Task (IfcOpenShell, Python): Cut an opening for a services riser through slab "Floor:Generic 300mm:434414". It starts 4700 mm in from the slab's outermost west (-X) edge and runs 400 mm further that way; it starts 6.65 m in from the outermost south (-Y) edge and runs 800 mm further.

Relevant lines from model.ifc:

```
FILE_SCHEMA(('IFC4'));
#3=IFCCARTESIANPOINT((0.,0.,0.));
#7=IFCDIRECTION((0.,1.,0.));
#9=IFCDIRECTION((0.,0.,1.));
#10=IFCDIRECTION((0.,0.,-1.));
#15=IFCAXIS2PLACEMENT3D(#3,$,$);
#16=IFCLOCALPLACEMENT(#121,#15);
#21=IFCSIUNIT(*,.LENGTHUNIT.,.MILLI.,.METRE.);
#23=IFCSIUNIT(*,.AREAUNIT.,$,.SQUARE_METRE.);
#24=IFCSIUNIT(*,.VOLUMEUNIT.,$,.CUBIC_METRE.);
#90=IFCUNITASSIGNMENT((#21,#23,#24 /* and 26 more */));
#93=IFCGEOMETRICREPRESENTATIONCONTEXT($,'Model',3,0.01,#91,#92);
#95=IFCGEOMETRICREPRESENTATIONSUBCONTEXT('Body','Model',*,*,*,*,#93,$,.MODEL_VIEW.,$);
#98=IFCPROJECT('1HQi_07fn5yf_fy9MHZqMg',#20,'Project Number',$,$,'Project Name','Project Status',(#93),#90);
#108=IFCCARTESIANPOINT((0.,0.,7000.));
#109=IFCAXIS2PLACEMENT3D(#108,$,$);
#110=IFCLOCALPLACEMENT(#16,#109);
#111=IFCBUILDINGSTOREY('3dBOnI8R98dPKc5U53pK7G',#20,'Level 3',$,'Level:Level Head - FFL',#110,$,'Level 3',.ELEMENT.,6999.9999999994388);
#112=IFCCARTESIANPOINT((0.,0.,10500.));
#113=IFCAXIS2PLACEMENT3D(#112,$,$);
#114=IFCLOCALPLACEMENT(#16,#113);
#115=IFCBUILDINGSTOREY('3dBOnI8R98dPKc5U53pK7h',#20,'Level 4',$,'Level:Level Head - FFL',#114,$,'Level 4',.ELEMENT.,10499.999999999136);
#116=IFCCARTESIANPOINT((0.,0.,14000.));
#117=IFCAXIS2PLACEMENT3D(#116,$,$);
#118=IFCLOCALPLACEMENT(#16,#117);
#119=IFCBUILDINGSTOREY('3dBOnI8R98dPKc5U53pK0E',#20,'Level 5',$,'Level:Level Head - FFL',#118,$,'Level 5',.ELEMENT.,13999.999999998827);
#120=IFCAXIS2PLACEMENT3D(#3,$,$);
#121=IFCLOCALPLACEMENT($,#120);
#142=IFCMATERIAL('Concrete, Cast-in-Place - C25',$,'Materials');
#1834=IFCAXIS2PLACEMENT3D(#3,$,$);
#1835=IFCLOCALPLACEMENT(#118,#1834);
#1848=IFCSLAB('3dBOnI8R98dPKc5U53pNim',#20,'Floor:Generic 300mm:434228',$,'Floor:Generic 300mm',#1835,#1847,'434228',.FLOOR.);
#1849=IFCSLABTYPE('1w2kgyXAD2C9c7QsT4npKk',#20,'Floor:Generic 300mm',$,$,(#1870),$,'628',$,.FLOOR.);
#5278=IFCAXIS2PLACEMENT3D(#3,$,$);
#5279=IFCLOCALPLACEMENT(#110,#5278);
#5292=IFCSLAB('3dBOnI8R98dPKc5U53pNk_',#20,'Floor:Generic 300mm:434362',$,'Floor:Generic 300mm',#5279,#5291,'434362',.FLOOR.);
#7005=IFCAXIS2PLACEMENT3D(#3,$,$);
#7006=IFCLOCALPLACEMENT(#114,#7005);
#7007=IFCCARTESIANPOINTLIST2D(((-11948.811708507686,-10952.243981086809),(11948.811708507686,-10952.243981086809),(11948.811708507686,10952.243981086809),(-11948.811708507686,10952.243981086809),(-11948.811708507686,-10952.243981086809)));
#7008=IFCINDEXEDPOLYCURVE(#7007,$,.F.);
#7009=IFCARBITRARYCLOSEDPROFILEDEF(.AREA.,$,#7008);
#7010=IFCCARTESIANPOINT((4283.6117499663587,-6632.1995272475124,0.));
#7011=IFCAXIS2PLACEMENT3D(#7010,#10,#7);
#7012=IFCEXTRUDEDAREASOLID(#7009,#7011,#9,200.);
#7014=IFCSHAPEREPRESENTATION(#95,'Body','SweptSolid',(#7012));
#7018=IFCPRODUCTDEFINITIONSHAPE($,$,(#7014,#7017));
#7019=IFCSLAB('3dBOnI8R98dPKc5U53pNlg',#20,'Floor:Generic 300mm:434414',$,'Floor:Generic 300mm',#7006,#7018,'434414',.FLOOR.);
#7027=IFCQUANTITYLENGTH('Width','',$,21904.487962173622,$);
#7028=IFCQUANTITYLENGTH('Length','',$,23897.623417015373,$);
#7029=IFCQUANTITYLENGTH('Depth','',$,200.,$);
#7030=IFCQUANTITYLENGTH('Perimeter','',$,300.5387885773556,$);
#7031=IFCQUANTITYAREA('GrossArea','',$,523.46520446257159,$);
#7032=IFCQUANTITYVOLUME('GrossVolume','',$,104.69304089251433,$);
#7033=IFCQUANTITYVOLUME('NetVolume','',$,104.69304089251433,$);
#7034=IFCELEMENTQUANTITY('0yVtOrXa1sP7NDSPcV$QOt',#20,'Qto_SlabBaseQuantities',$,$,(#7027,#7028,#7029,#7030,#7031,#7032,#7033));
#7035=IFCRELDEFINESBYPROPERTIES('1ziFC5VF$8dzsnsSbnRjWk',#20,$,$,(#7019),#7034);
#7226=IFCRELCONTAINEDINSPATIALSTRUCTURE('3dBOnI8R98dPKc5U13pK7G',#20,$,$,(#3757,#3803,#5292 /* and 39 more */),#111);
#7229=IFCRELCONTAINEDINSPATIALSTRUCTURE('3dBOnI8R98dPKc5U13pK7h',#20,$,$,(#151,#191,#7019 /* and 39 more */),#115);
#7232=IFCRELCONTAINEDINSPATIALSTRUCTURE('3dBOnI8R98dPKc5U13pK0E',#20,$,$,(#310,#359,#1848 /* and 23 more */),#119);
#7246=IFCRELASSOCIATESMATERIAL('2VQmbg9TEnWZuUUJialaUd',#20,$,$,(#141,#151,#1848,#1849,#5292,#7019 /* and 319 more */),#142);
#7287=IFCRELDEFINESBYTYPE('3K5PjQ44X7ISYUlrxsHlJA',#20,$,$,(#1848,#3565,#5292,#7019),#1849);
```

```python
import numpy as np
import ifcopenshell
import ifcopenshell.api.feature
import ifcopenshell.api.geometry
import ifcopenshell.api.pset
import ifcopenshell.api.root
import ifcopenshell.geom
import ifcopenshell.util.element
import ifcopenshell.util.placement
import ifcopenshell.util.representation
import ifcopenshell.util.shape
import ifcopenshell.util.unit

model = ifcopenshell.open("model.ifc")
unit_scale = ifcopenshell.util.unit.calculate_unit_scale(model)
volume_scale = ifcopenshell.util.unit.calculate_unit_scale(model, "VOLUMEUNIT")
settings = ifcopenshell.geom.settings()


def volume(element):
    """Net volume in cubic metres, openings subtracted."""
    shape = ifcopenshell.geom.create_shape(settings, element)
    return ifcopenshell.util.shape.get_volume(shape.geometry)


slab = model.by_guid("3dBOnI8R98dPKc5U53pNlg")
before = volume(slab)

# Extent in the slab's own axes, in metres. The edges named are its -X and -Y sides.
slab_shape = ifcopenshell.geom.create_shape(settings, slab)
vertices = ifcopenshell.util.shape.get_vertices(slab_shape.geometry)
x_min, y_min, bottom = vertices.min(axis=0)
top = vertices[:, 2].max()

opening = ifcopenshell.api.root.create_entity(model, ifc_class="IfcOpeningElement", name="Services riser opening", predefined_type="OPENING")
context = ifcopenshell.util.representation.get_context(model, "Model", "Body", "MODEL_VIEW")
width, depth = 0.4, 0.8
outline = [(0.0, 0.0), (width, 0.0), (width, depth), (0.0, depth), (0.0, 0.0)]
# Overshoot both faces by 50 mm so the cut is clean.
shape = ifcopenshell.api.geometry.add_slab_representation(
    model, context=context, depth=top - bottom + 0.1, polyline=outline
)
ifcopenshell.api.geometry.assign_representation(model, product=opening, representation=shape)

matrix = ifcopenshell.util.placement.get_local_placement(slab.ObjectPlacement)
matrix[:, 3] = matrix @ np.append(np.array([x_min + 4.7, y_min + 6.65, bottom - 0.05]) / unit_scale, 1.0)
ifcopenshell.api.geometry.edit_object_placement(model, product=opening, matrix=matrix, is_si=False)
ifcopenshell.api.feature.add_feature(model, feature=opening, element=slab)

after = volume(slab)

# Update the slab's stored quantities.
qto = model.by_id(ifcopenshell.util.element.get_pset(slab, "Qto_SlabBaseQuantities", should_inherit=False)["id"])
ifcopenshell.api.pset.edit_qto(model, qto=qto, properties={"NetVolume": after / volume_scale})

print(f"slab volume {before:.3f} -> {after:.3f} m3")

model.write("model_updated.ifc")
```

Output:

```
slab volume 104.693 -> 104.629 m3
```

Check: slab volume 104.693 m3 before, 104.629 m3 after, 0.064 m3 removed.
